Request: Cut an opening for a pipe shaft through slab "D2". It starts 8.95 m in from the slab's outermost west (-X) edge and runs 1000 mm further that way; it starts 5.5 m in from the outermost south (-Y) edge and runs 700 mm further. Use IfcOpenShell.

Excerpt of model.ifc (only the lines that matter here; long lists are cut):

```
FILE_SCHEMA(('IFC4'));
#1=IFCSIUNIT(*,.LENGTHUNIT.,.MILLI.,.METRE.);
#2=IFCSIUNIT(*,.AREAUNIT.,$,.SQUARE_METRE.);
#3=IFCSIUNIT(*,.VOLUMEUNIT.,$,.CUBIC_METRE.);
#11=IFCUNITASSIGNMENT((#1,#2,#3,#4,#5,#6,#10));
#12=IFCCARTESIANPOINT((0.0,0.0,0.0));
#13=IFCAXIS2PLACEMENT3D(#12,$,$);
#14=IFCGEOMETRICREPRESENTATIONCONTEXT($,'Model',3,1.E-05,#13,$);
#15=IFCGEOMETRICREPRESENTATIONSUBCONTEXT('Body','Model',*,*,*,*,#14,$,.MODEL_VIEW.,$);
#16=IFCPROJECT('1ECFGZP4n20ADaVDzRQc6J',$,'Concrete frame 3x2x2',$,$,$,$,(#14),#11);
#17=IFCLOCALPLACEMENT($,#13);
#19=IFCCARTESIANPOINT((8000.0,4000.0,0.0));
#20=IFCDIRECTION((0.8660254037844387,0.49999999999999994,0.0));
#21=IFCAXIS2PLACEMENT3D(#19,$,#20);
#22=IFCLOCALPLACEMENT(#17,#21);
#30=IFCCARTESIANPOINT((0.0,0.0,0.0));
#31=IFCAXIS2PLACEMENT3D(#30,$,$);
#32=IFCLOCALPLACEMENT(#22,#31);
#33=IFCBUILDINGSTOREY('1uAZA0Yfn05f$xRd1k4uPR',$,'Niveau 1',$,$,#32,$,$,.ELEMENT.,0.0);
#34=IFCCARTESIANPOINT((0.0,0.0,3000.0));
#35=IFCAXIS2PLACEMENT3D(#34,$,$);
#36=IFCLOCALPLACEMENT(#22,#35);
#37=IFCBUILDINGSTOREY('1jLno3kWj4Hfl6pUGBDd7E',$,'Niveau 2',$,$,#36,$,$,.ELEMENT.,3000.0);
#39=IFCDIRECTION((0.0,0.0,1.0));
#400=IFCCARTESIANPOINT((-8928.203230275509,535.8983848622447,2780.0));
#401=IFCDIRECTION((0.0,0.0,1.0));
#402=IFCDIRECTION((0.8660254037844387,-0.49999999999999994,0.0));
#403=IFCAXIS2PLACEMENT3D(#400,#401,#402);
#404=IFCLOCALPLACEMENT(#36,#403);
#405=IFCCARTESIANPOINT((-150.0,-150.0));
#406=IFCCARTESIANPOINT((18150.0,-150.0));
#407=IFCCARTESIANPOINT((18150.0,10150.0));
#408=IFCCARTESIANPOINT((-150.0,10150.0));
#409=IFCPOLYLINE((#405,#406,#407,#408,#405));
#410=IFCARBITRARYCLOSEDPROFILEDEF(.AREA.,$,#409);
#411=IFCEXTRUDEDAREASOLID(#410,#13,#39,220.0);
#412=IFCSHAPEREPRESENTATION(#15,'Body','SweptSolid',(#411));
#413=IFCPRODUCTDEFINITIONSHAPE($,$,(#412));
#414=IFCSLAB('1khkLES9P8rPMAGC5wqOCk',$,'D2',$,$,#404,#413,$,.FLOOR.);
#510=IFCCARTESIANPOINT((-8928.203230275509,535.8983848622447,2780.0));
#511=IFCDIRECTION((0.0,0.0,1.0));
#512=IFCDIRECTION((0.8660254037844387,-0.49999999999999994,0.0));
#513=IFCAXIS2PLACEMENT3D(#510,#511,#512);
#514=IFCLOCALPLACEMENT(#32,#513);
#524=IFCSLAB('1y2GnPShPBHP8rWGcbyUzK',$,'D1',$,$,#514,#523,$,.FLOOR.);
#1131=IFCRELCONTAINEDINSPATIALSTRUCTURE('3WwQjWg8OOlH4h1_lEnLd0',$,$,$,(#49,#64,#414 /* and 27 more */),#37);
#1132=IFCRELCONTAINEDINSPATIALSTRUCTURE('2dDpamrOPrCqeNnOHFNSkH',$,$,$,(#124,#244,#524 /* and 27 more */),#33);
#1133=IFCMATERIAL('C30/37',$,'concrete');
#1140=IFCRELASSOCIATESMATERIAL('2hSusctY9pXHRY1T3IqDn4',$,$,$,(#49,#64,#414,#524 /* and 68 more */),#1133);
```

```python
import numpy as np
import ifcopenshell
import ifcopenshell.api.feature
import ifcopenshell.api.geometry
import ifcopenshell.api.root
import ifcopenshell.geom
import ifcopenshell.util.placement
import ifcopenshell.util.representation
import ifcopenshell.util.shape
import ifcopenshell.util.unit

model = ifcopenshell.open("model.ifc")
unit_scale = ifcopenshell.util.unit.calculate_unit_scale(model)
settings = ifcopenshell.geom.settings()


def volume(element):
    """Net volume in cubic metres, openings subtracted."""
    shape = ifcopenshell.geom.create_shape(settings, element)
    return ifcopenshell.util.shape.get_volume(shape.geometry)


slab = model.by_id(414)
before = volume(slab)

# Extent in the slab's own axes, in metres. The edges named are its -X and -Y sides.
slab_shape = ifcopenshell.geom.create_shape(settings, slab)
vertices = ifcopenshell.util.shape.get_vertices(slab_shape.geometry)
x_min, y_min, bottom = vertices.min(axis=0)
top = vertices[:, 2].max()

opening = ifcopenshell.api.root.create_entity(model, ifc_class="IfcOpeningElement", name="Pipe shaft opening", predefined_type="OPENING")
context = ifcopenshell.util.representation.get_context(model, "Model", "Body", "MODEL_VIEW")
width, depth = 1, 0.7
outline = [(0.0, 0.0), (width, 0.0), (width, depth), (0.0, depth), (0.0, 0.0)]
# Overshoot both faces by 50 mm so the cut is clean.
shape = ifcopenshell.api.geometry.add_slab_representation(
    model, context=context, depth=top - bottom + 0.1, polyline=outline
)
ifcopenshell.api.geometry.assign_representation(model, product=opening, representation=shape)

matrix = ifcopenshell.util.placement.get_local_placement(slab.ObjectPlacement)
matrix[:, 3] = matrix @ np.append(np.array([x_min + 8.95, y_min + 5.5, bottom - 0.05]) / unit_scale, 1.0)
ifcopenshell.api.geometry.edit_object_placement(model, product=opening, matrix=matrix, is_si=False)
ifcopenshell.api.feature.add_feature(model, feature=opening, element=slab)

after = volume(slab)

print(f"slab volume {before:.3f} -> {after:.3f} m3")

model.write("model_edited.ifc")
```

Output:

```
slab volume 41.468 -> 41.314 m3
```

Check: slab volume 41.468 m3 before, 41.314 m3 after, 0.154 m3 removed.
